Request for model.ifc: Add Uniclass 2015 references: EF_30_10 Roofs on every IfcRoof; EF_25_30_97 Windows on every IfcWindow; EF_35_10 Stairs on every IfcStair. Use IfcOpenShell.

First a look at what the model holds.

```python
import ifcopenshell

model = ifcopenshell.open("model.ifc")
print(model.schema)
print("classifications:", [c.Name for c in model.by_type("IfcClassification")])
for ifc_class in ("IfcDoor", "IfcRoof", "IfcStair", "IfcWall", "IfcWindow"):
    print(ifc_class, len(model.by_type(ifc_class)))
```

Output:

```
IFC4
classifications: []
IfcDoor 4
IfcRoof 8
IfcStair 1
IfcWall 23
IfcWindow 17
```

```python
import ifcopenshell
import ifcopenshell.api.classification

model = ifcopenshell.open("model.ifc")

system = ifcopenshell.api.classification.add_classification(model, classification="Uniclass 2015")

codes = {
    "IfcRoof": ("EF_30_10", "Roofs"),
    "IfcWindow": ("EF_25_30_97", "Windows"),
    "IfcStair": ("EF_35_10", "Stairs"),
}
for ifc_class, (code, name) in codes.items():
    products = model.by_type(ifc_class)
    ifcopenshell.api.classification.add_reference(
        model, products=products, classification=system, identification=code, name=name
    )
    print(code, len(products))

model.write("model_rev.ifc")
```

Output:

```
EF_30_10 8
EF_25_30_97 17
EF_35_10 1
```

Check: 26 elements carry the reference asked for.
